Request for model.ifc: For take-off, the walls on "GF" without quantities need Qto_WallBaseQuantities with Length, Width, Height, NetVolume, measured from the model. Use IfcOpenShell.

First a look at what the model holds.

```python
import ifcopenshell
import ifcopenshell.util.element
import ifcopenshell.util.unit

model = ifcopenshell.open("model.ifc")
print(model.schema)
for unit_type in ("LENGTHUNIT", "AREAUNIT", "VOLUMEUNIT"):
    print(unit_type, ifcopenshell.util.unit.calculate_unit_scale(model, unit_type))
storey = next(s for s in model.by_type("IfcBuildingStorey") if s.Name == "GF")
walls = [e for e in ifcopenshell.util.element.get_decomposition(storey) if e.is_a("IfcWall")]
for e in sorted(walls, key=lambda e: e.id()):
    print(e.id(), e.is_a(), e.Name, list(ifcopenshell.util.element.get_psets(e, qtos_only=True)), sep=" | ")
```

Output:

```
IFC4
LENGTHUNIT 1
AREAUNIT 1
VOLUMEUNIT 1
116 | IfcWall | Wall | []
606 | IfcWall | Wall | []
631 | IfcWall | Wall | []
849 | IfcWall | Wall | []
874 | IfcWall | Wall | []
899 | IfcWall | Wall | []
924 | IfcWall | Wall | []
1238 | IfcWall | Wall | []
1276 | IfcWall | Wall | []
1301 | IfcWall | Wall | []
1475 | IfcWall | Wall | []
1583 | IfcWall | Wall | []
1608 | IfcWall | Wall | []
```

```python
import ifcopenshell
import ifcopenshell.api.pset
import ifcopenshell.geom
import ifcopenshell.util.element
import ifcopenshell.util.shape
import ifcopenshell.util.unit

model = ifcopenshell.open("model.ifc")
unit_scale = ifcopenshell.util.unit.calculate_unit_scale(model)
volume_scale = ifcopenshell.util.unit.calculate_unit_scale(model, "VOLUMEUNIT")
settings = ifcopenshell.geom.settings()

storey = next(s for s in model.by_type("IfcBuildingStorey") if s.Name == "GF")
walls = [e for e in ifcopenshell.util.element.get_decomposition(storey) if e.is_a("IfcWall")]

for e in sorted(walls, key=lambda e: e.id()):
    if ifcopenshell.util.element.get_psets(e, qtos_only=True, should_inherit=False):
        continue
    # Geometry comes back in metres, in the element's own axes.
    shape = ifcopenshell.geom.create_shape(settings, e)
    values = {
        "Length": ifcopenshell.util.shape.get_x(shape.geometry) / unit_scale,
        "Width": ifcopenshell.util.shape.get_y(shape.geometry) / unit_scale,
        "Height": ifcopenshell.util.shape.get_z(shape.geometry) / unit_scale,
        "NetVolume": ifcopenshell.util.shape.get_volume(shape.geometry) / volume_scale,
    }
    qto = ifcopenshell.api.pset.add_qto(model, product=e, name="Qto_WallBaseQuantities")
    ifcopenshell.api.pset.edit_qto(model, qto=qto, properties=values)
    print(e.id(), {k: round(v, 3) for k, v in values.items()})

model.write("model_rev.ifc")
```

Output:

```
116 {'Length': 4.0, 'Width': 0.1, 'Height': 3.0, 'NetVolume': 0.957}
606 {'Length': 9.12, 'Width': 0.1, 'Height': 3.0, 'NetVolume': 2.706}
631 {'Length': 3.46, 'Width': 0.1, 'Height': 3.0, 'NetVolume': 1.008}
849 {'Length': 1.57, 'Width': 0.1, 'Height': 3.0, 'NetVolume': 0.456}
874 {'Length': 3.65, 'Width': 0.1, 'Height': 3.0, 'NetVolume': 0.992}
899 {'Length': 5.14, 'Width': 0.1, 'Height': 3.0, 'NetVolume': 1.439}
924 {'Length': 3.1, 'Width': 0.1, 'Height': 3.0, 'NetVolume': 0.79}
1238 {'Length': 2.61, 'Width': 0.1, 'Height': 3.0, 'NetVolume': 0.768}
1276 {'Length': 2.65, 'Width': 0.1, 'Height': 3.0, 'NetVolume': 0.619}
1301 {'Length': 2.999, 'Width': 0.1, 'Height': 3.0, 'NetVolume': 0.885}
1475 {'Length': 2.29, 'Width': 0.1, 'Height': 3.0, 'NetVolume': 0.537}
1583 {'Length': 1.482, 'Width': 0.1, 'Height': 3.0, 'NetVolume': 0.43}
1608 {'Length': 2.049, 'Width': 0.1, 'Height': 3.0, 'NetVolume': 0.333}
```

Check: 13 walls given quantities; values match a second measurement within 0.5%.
